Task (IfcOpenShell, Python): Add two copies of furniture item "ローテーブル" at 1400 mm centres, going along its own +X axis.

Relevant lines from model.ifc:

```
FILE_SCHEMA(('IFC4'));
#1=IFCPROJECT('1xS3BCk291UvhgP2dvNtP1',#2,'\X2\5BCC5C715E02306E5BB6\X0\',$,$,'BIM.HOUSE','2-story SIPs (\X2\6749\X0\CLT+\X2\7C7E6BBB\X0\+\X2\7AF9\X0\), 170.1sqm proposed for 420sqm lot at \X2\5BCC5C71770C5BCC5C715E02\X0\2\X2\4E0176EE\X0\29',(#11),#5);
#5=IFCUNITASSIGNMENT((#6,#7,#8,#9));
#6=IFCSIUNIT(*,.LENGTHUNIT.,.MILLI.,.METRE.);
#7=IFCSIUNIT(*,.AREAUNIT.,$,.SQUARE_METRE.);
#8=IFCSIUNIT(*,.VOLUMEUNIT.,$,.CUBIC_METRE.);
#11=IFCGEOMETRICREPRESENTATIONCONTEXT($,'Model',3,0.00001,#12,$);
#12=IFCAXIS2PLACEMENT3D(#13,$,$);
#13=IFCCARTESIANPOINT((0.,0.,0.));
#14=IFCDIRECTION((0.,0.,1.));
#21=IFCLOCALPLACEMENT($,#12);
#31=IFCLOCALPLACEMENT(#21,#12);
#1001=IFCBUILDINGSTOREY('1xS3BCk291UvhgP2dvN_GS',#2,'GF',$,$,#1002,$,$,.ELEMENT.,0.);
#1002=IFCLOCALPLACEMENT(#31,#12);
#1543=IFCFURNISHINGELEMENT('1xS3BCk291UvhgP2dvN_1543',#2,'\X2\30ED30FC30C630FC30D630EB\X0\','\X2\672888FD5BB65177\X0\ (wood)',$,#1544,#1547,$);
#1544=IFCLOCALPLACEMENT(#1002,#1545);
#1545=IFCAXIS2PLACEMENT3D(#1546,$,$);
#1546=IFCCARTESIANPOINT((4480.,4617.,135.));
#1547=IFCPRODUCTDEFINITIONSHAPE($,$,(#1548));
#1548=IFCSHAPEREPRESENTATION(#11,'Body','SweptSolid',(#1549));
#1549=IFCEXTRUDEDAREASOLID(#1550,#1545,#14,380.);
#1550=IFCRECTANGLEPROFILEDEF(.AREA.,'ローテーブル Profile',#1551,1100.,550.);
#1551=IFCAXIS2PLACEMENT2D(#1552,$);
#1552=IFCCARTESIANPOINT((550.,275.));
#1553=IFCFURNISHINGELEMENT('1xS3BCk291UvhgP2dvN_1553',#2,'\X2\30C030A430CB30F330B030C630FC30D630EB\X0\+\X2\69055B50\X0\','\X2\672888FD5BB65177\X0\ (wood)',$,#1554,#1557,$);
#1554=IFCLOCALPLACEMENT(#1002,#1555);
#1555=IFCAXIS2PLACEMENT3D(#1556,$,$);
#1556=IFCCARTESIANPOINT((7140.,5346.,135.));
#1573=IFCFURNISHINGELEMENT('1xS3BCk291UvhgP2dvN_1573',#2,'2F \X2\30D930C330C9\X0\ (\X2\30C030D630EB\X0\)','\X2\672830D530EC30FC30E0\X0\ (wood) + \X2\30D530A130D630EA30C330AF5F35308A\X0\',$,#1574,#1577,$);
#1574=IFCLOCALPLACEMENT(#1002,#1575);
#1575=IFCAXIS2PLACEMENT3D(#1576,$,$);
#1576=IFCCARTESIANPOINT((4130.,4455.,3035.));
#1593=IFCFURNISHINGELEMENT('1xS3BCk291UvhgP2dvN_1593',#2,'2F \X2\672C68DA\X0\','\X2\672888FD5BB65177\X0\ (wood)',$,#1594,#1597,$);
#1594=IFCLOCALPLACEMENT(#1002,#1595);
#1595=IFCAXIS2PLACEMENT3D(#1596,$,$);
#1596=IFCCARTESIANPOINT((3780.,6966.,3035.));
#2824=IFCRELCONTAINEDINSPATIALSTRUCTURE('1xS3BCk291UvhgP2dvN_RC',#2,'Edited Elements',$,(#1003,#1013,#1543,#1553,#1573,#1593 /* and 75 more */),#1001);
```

```python
import ifcopenshell
import ifcopenshell.api.geometry
import ifcopenshell.api.root
import ifcopenshell.util.element
import ifcopenshell.util.placement

model = ifcopenshell.open("model.ifc")


def reuse_history(source, copy):
    """copy_class also copies each property set's owner history, people and application; keep the originals."""
    for rel in copy.IsDefinedBy:
        if rel.is_a("IfcRelDefinesByProperties") and (history := rel.RelatingPropertyDefinition.OwnerHistory):
            rel.RelatingPropertyDefinition.OwnerHistory = source.OwnerHistory
            ifcopenshell.util.element.remove_deep2(model, history)


source = model.by_guid("1xS3BCk291UvhgP2dvN_1543")
base = ifcopenshell.util.placement.get_local_placement(source.ObjectPlacement)
step = base[:3, 0] * 1400.0

for i in range(1, 3):
    copy = ifcopenshell.api.root.copy_class(model, product=source)
    copy.Representation = ifcopenshell.util.element.copy_deep(
        model, source.Representation, exclude=["IfcGeometricRepresentationContext", "IfcRepresentationMap"]
    )
    reuse_history(source, copy)
    matrix = base.copy()
    matrix[:3, 3] += i * step
    print("added at", matrix[:3, 3].round(3) + 0.0)
    ifcopenshell.api.geometry.edit_object_placement(model, product=copy, matrix=matrix, is_si=False)

model.write("model-out.ifc")
```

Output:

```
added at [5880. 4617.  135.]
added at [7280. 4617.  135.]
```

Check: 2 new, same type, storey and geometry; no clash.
